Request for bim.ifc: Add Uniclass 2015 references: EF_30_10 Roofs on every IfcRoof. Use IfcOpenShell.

First a look at what the model holds.

```python
import ifcopenshell

model = ifcopenshell.open("bim.ifc")
print(model.schema)
print("classifications:", [c.Name for c in model.by_type("IfcClassification")])
for ifc_class in ("IfcDoor", "IfcRoof", "IfcStair", "IfcWall", "IfcWindow"):
    print(ifc_class, len(model.by_type(ifc_class)))
```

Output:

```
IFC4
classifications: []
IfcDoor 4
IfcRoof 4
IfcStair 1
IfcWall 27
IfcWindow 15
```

```python
import ifcopenshell
import ifcopenshell.api.classification

model = ifcopenshell.open("bim.ifc")

system = ifcopenshell.api.classification.add_classification(model, classification="Uniclass 2015")

codes = {
    "IfcRoof": ("EF_30_10", "Roofs"),
}
for ifc_class, (code, name) in codes.items():
    products = model.by_type(ifc_class)
    ifcopenshell.api.classification.add_reference(
        model, products=products, classification=system, identification=code, name=name
    )
    print(code, len(products))

model.write("bim_rev.ifc")
```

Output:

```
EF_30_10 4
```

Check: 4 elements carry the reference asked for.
